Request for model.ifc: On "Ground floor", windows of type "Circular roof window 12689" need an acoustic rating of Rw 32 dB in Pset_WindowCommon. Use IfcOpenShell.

First a look at what the model holds.

```python
import ifcopenshell
import ifcopenshell.util.element

model = ifcopenshell.open("model.ifc")
print(model.schema)
storey = next(s for s in model.by_type("IfcBuildingStorey") if s.Name == "Ground floor")
windows = [e for e in ifcopenshell.util.element.get_decomposition(storey) if e.is_a("IfcWindow")]
seen = {}
for e in windows:
    element_type = ifcopenshell.util.element.get_type(e)
    key = (element_type.Name if element_type != e and element_type else None, ifcopenshell.util.element.get_pset(e, "Pset_WindowCommon", "AcousticRating"))
    seen[key] = seen.get(key, 0) + 1
for (name, value), count in sorted(seen.items(), key=str):
    print(count, "x", name, "|", value)
```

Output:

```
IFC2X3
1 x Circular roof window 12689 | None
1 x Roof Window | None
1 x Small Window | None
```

```python
import ifcopenshell
import ifcopenshell.api.pset
import ifcopenshell.util.element

model = ifcopenshell.open("model.ifc")

storey = next(s for s in model.by_type("IfcBuildingStorey") if s.Name == "Ground floor")
windows = [e for e in ifcopenshell.util.element.get_decomposition(storey) if e.is_a("IfcWindow")]

count = 0
for e in windows:
    element_type = ifcopenshell.util.element.get_type(e)
    if element_type in (None, e) or element_type.Name != "Circular roof window 12689":
        continue
    # add_pset returns the element's existing set when there is one.
    pset = ifcopenshell.api.pset.add_pset(model, product=e, name="Pset_WindowCommon")
    ifcopenshell.api.pset.edit_pset(model, pset=pset, properties={"AcousticRating": "Rw 32 dB"})
    count += 1

print(count, "windows updated")

model.write("model_updated.ifc")
```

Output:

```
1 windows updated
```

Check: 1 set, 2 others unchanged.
